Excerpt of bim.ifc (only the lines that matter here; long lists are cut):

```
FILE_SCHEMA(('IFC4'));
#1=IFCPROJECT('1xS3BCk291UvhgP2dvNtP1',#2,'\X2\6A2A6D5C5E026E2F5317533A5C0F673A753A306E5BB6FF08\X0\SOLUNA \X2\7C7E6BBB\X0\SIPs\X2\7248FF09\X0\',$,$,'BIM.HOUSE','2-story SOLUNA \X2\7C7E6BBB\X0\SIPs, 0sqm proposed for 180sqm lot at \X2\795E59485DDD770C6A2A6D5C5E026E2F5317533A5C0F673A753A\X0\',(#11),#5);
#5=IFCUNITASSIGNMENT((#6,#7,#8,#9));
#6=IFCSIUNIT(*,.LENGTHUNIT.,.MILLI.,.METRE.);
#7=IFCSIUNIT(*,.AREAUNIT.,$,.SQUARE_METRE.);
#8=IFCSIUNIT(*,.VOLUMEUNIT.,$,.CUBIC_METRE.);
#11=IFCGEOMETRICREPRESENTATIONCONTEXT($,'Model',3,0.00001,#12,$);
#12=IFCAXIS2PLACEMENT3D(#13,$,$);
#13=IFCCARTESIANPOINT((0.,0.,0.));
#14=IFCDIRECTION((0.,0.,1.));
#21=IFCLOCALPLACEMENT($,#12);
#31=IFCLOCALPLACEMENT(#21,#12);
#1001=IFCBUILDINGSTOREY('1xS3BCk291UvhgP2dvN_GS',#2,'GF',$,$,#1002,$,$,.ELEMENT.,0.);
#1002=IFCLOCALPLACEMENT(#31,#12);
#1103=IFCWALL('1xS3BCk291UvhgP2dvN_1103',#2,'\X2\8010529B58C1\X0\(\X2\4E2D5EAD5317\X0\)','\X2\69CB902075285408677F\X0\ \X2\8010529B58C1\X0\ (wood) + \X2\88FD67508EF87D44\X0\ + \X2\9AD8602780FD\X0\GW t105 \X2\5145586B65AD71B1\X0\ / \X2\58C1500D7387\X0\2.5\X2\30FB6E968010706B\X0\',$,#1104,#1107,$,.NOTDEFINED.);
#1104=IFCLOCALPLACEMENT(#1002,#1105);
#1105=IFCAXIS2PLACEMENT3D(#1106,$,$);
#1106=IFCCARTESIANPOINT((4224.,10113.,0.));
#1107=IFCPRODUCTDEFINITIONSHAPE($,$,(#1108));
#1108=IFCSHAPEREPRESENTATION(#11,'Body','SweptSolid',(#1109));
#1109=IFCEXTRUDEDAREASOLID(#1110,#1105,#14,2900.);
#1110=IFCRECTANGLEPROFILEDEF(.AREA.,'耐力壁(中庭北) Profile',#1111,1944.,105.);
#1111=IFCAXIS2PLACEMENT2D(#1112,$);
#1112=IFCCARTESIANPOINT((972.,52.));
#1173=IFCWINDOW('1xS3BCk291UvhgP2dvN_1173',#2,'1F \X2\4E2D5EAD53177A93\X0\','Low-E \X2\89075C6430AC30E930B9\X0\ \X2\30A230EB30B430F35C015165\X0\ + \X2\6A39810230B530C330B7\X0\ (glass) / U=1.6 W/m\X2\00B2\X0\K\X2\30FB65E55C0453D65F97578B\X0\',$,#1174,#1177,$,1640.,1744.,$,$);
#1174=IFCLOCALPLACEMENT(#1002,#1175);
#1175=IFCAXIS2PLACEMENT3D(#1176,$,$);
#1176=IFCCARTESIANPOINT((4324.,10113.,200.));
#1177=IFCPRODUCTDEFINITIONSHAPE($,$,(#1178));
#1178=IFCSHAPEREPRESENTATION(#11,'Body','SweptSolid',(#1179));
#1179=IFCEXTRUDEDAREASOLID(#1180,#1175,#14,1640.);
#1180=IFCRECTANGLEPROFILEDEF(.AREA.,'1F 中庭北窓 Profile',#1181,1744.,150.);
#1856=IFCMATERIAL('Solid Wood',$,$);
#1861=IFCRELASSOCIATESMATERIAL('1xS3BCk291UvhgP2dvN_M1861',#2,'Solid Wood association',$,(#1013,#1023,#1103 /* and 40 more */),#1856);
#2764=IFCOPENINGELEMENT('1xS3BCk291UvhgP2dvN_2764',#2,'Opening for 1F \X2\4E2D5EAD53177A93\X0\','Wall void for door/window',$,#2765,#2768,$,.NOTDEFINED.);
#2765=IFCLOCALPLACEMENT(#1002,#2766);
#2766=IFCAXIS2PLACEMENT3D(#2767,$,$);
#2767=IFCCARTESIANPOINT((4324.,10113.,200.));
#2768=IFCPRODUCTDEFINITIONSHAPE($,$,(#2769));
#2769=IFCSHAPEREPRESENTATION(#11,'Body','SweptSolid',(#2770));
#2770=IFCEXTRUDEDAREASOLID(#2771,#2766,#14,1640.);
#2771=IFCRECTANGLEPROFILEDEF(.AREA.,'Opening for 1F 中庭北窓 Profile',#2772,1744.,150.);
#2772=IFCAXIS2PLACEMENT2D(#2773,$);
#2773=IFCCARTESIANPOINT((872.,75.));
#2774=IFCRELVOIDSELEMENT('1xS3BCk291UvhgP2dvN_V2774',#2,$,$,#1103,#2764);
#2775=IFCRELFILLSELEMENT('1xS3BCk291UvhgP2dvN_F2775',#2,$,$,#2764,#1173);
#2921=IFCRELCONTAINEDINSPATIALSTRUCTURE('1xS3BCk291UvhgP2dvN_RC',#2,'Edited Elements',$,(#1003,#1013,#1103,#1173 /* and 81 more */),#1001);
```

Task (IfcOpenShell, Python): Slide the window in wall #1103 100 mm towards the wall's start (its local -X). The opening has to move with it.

```python
import ifcopenshell
import ifcopenshell.api.geometry
import ifcopenshell.util.placement
import ifcopenshell.util.unit

model = ifcopenshell.open("bim.ifc")
unit_scale = ifcopenshell.util.unit.calculate_unit_scale(model)

window = model.by_guid("1xS3BCk291UvhgP2dvN_1173")
opening = window.FillsVoids[0].RelatingOpeningElement
wall = opening.VoidsElements[0].RelatingBuildingElement

wall_matrix = ifcopenshell.util.placement.get_local_placement(wall.ObjectPlacement)
shift = wall_matrix[:3, 0] * -0.1 / unit_scale
before = ifcopenshell.util.placement.get_local_placement(window.ObjectPlacement)[:3, 3].copy()

# The window is not placed relative to its opening, so move both.
for product in (opening, window):
    matrix = ifcopenshell.util.placement.get_local_placement(product.ObjectPlacement)
    matrix[:3, 3] += shift
    ifcopenshell.api.geometry.edit_object_placement(model, product=product, matrix=matrix, is_si=False)

after = ifcopenshell.util.placement.get_local_placement(window.ObjectPlacement)[:3, 3]
print("window moved by", (after - before).round(3) + 0.0)

model.write("bim_edited.ifc")
```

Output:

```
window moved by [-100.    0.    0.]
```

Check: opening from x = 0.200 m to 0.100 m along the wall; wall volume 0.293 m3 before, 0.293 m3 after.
